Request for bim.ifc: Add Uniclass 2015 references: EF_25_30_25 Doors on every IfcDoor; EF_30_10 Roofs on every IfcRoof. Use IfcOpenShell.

First a look at what the model holds.

```python
import ifcopenshell

model = ifcopenshell.open("bim.ifc")
print(model.schema)
print("classifications:", [c.Name for c in model.by_type("IfcClassification")])
for ifc_class in ("IfcDoor", "IfcRoof", "IfcStair", "IfcWall", "IfcWindow"):
    print(ifc_class, len(model.by_type(ifc_class)))
```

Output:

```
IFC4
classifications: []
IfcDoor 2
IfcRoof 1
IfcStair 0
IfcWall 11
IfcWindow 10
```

```python
import ifcopenshell
import ifcopenshell.api.classification

model = ifcopenshell.open("bim.ifc")

system = ifcopenshell.api.classification.add_classification(model, classification="Uniclass 2015")

codes = {
    "IfcDoor": ("EF_25_30_25", "Doors"),
    "IfcRoof": ("EF_30_10", "Roofs"),
}
for ifc_class, (code, name) in codes.items():
    products = model.by_type(ifc_class)
    ifcopenshell.api.classification.add_reference(
        model, products=products, classification=system, identification=code, name=name
    )
    print(code, len(products))

model.write("bim_edited.ifc")
```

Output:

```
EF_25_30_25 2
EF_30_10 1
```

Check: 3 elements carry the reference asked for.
